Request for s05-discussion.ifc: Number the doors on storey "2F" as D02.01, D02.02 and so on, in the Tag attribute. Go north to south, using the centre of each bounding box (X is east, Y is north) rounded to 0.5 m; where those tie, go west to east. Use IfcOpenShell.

First a look at what the model holds.

```python
import ifcopenshell
import ifcopenshell.util.element
import ifcopenshell.util.placement

model = ifcopenshell.open("s05-discussion.ifc")
print(model.schema)
storey = next(s for s in model.by_type("IfcBuildingStorey") if s.Name == "2F")
doors = [e for e in ifcopenshell.util.element.get_decomposition(storey) if e.is_a("IfcDoor")]
for e in sorted(doors, key=lambda e: e.id()):
    origin = ifcopenshell.util.placement.get_local_placement(e.ObjectPlacement)[:3, 3]
    print(e.id(), e.Tag, e.Name, origin.round(2) + 0.0, sep=" | ")
```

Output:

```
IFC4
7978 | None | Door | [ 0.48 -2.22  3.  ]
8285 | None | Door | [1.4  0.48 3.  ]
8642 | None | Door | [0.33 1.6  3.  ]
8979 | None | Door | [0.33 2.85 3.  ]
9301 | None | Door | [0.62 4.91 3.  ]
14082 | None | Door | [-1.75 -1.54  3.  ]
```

```python
import ifcopenshell
import ifcopenshell.geom
import ifcopenshell.util.element
import ifcopenshell.util.shape

model = ifcopenshell.open("s05-discussion.ifc")
settings = ifcopenshell.geom.settings()
settings.set("use-world-coords", True)


def centre(element):
    shape = ifcopenshell.geom.create_shape(settings, element)
    return ifcopenshell.util.shape.get_bbox_centroid(shape.geometry)


storey = next(s for s in model.by_type("IfcBuildingStorey") if s.Name == "2F")
doors = [e for e in ifcopenshell.util.element.get_decomposition(storey) if e.is_a("IfcDoor")]

# Insertion points can sit at a corner or the storey origin, so sort by the geometry (in metres).
centres = {e: centre(e) for e in doors}
doors.sort(key=lambda e: (-round(centres[e][1] / 0.5), centres[e][0]))

for i, e in enumerate(doors, start=1):
    number = f"D02.{i:02d}"
    e.Tag = number
    print(e.id(), number)

model.write("s05-discussion_rev.ifc")
```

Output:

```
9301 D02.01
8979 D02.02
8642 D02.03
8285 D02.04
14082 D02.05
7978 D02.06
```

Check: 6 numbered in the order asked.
